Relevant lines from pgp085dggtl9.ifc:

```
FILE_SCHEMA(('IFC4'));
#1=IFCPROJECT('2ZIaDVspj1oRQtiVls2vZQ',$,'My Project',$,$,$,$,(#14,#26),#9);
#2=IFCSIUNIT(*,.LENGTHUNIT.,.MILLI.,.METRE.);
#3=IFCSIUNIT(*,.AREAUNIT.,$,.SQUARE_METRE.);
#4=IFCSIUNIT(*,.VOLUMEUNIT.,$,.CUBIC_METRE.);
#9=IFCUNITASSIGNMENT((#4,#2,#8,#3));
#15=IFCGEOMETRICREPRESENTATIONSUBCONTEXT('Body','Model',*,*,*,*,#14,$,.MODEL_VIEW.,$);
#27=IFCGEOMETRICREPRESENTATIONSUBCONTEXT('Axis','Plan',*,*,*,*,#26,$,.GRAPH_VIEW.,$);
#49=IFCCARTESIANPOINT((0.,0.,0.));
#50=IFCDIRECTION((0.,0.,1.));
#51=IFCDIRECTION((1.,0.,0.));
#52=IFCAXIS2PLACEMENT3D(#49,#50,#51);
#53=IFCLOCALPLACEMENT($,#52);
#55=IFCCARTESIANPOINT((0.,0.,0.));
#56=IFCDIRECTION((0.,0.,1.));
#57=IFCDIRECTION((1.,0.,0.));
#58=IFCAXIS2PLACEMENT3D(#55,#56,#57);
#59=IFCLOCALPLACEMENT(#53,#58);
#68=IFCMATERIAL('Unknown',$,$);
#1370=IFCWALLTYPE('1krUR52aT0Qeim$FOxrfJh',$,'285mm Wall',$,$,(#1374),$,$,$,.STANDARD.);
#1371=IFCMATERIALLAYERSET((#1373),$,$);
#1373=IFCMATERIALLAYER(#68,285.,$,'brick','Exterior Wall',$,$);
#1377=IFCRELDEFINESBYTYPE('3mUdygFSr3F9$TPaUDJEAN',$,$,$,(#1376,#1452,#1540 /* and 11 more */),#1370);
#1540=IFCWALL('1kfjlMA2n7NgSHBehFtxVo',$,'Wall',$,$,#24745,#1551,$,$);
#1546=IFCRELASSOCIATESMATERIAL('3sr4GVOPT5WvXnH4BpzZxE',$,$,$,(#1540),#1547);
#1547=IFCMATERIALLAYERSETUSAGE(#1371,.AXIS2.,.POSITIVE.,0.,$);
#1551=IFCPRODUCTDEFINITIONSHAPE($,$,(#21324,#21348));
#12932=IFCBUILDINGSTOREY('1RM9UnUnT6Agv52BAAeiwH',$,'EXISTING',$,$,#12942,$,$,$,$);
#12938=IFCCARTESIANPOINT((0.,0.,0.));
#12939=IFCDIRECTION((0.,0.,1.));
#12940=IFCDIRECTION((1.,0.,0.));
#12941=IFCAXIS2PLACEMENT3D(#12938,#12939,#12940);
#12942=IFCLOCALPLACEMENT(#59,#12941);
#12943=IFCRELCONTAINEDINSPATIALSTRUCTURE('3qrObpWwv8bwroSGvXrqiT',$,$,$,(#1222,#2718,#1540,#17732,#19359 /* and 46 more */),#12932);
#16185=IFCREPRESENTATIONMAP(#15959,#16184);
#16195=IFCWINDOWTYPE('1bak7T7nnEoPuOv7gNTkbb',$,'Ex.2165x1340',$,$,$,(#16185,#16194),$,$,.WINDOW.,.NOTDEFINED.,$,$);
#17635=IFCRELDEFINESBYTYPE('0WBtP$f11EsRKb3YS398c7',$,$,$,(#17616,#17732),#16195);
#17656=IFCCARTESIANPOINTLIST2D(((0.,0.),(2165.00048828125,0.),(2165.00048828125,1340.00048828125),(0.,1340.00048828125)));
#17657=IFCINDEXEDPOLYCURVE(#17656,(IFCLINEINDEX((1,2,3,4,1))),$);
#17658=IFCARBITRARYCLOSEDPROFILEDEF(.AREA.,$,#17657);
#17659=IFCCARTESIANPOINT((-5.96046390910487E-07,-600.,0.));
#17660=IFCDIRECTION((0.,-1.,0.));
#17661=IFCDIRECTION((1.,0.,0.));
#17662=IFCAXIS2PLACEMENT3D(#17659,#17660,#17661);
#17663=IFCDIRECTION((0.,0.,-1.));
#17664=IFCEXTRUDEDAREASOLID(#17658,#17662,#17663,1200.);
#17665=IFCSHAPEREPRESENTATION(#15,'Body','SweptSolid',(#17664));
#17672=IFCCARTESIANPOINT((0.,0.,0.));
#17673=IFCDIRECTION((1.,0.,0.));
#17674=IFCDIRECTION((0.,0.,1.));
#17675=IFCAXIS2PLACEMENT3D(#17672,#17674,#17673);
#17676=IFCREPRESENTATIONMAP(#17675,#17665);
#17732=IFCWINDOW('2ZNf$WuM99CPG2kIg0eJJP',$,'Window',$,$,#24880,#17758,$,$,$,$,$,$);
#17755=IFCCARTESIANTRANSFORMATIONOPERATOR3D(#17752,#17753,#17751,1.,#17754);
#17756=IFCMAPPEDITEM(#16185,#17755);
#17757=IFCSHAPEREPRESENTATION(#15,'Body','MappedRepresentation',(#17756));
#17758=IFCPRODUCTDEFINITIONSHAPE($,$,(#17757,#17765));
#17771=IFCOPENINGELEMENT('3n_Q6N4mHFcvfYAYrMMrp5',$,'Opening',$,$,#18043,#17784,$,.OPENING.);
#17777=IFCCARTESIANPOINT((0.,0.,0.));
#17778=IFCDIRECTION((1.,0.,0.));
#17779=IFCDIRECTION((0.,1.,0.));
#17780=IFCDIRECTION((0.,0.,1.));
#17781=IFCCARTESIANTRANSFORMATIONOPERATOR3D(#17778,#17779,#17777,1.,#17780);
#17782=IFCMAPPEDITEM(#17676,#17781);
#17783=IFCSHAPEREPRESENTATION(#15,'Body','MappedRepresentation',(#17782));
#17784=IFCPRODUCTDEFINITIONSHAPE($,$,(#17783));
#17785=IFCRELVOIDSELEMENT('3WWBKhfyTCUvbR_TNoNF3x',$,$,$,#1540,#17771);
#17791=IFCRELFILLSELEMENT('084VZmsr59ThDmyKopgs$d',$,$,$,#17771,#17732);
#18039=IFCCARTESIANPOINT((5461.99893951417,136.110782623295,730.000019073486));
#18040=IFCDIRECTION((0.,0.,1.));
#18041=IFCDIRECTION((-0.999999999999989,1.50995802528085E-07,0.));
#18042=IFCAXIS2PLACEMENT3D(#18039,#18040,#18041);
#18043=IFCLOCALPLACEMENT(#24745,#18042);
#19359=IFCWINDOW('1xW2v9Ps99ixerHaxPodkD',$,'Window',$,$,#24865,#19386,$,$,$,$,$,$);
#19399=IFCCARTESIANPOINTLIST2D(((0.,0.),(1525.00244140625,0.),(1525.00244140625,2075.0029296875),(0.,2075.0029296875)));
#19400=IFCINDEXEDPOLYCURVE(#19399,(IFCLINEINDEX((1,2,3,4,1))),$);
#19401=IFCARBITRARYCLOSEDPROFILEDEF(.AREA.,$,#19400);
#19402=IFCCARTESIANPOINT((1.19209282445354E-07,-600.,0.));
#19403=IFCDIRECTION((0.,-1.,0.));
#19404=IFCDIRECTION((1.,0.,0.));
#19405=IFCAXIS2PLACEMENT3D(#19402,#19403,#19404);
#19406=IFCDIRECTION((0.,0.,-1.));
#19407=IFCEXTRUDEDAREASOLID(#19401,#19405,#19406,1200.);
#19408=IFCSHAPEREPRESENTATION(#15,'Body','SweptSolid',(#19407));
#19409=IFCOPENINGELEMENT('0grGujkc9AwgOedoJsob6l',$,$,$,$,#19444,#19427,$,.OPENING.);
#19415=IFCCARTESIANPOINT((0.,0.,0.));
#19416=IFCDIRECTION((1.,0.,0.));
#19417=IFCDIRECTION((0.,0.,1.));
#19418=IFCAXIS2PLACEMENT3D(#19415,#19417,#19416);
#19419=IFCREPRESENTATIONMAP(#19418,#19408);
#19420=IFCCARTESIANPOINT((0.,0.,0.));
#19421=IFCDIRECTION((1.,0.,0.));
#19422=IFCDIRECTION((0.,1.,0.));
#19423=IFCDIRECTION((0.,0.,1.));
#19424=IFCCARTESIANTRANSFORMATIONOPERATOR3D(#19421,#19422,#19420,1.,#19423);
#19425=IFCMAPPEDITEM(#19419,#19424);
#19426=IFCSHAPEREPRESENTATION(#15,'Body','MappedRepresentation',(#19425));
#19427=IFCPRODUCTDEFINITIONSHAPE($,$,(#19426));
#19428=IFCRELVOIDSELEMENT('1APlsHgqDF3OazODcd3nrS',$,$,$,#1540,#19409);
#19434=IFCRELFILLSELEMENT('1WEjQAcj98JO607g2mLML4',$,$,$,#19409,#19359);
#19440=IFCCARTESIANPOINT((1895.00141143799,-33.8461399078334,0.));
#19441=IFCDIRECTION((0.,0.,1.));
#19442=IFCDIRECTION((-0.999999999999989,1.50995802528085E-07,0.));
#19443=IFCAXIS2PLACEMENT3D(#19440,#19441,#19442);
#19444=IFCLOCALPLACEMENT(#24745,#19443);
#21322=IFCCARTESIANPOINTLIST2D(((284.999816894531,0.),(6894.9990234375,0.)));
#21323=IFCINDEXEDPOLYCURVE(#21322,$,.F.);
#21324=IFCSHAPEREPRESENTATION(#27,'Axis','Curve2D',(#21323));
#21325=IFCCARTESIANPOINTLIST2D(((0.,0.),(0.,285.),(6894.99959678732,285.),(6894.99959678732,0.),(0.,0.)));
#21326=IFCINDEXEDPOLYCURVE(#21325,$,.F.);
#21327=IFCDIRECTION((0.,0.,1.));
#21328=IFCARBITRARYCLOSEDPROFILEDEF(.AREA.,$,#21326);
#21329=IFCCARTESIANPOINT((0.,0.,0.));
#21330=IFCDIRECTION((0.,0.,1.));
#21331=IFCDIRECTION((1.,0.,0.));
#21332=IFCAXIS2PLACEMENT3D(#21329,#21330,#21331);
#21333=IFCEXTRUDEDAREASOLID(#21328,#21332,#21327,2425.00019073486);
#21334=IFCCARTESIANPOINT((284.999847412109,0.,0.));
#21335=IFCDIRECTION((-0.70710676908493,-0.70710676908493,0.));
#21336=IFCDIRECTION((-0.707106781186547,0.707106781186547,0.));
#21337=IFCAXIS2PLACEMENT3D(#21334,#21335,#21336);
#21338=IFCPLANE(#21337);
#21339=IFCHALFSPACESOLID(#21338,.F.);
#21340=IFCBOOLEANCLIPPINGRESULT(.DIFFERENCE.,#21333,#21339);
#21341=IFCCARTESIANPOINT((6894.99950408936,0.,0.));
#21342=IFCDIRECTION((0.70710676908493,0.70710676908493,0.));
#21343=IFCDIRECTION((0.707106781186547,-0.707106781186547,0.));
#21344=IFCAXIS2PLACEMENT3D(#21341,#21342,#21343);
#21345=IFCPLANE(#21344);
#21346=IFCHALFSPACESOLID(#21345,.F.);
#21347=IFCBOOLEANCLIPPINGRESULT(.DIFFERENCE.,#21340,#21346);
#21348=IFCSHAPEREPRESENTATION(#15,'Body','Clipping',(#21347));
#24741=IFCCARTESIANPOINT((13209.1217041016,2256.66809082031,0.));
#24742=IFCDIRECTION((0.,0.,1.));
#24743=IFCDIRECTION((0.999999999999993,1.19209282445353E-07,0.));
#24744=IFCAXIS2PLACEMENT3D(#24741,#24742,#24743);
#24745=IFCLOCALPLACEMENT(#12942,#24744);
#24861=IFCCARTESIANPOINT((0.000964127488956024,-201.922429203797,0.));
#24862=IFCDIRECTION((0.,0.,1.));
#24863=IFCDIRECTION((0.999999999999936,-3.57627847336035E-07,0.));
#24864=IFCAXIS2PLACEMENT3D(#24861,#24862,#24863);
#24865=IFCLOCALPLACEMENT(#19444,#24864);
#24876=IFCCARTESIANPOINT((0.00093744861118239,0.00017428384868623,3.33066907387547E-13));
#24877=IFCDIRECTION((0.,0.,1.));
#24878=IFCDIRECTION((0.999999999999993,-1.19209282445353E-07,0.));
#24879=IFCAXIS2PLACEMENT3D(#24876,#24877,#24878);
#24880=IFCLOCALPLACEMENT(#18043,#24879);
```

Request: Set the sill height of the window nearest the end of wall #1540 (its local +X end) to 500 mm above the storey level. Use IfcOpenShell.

```python
import numpy as np
import ifcopenshell
import ifcopenshell.api.geometry
import ifcopenshell.geom
import ifcopenshell.util.element
import ifcopenshell.util.placement
import ifcopenshell.util.shape
import ifcopenshell.util.unit

model = ifcopenshell.open("pgp085dggtl9.ifc")
unit_scale = ifcopenshell.util.unit.calculate_unit_scale(model)

window = model.by_id(17732)
opening = window.FillsVoids[0].RelatingOpeningElement
storey = ifcopenshell.util.element.get_container(window, ifc_class="IfcBuildingStorey")
level = ifcopenshell.util.placement.get_local_placement(storey.ObjectPlacement)[2, 3]

# The opening's origin need not be at the sill, so measure its lowest point.
shape = ifcopenshell.geom.create_shape(ifcopenshell.geom.settings(), opening)
bottom = ifcopenshell.util.shape.get_shape_bottom_elevation(shape, shape.geometry) / unit_scale
dz = level + 0.5 / unit_scale - bottom

shift = np.array([0.0, 0.0, dz])
# The window is placed relative to its opening, so it follows when the opening moves.
matrix = ifcopenshell.util.placement.get_local_placement(opening.ObjectPlacement)
matrix[:3, 3] += shift
ifcopenshell.api.geometry.edit_object_placement(
    model, product=opening, matrix=matrix, is_si=False, should_transform_children=True
)

print(f"moved by {dz * unit_scale:+.3f} m")

model.write("pgp085dggtl9_v2.ifc")
```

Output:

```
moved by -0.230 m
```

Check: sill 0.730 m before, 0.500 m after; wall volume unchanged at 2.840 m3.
